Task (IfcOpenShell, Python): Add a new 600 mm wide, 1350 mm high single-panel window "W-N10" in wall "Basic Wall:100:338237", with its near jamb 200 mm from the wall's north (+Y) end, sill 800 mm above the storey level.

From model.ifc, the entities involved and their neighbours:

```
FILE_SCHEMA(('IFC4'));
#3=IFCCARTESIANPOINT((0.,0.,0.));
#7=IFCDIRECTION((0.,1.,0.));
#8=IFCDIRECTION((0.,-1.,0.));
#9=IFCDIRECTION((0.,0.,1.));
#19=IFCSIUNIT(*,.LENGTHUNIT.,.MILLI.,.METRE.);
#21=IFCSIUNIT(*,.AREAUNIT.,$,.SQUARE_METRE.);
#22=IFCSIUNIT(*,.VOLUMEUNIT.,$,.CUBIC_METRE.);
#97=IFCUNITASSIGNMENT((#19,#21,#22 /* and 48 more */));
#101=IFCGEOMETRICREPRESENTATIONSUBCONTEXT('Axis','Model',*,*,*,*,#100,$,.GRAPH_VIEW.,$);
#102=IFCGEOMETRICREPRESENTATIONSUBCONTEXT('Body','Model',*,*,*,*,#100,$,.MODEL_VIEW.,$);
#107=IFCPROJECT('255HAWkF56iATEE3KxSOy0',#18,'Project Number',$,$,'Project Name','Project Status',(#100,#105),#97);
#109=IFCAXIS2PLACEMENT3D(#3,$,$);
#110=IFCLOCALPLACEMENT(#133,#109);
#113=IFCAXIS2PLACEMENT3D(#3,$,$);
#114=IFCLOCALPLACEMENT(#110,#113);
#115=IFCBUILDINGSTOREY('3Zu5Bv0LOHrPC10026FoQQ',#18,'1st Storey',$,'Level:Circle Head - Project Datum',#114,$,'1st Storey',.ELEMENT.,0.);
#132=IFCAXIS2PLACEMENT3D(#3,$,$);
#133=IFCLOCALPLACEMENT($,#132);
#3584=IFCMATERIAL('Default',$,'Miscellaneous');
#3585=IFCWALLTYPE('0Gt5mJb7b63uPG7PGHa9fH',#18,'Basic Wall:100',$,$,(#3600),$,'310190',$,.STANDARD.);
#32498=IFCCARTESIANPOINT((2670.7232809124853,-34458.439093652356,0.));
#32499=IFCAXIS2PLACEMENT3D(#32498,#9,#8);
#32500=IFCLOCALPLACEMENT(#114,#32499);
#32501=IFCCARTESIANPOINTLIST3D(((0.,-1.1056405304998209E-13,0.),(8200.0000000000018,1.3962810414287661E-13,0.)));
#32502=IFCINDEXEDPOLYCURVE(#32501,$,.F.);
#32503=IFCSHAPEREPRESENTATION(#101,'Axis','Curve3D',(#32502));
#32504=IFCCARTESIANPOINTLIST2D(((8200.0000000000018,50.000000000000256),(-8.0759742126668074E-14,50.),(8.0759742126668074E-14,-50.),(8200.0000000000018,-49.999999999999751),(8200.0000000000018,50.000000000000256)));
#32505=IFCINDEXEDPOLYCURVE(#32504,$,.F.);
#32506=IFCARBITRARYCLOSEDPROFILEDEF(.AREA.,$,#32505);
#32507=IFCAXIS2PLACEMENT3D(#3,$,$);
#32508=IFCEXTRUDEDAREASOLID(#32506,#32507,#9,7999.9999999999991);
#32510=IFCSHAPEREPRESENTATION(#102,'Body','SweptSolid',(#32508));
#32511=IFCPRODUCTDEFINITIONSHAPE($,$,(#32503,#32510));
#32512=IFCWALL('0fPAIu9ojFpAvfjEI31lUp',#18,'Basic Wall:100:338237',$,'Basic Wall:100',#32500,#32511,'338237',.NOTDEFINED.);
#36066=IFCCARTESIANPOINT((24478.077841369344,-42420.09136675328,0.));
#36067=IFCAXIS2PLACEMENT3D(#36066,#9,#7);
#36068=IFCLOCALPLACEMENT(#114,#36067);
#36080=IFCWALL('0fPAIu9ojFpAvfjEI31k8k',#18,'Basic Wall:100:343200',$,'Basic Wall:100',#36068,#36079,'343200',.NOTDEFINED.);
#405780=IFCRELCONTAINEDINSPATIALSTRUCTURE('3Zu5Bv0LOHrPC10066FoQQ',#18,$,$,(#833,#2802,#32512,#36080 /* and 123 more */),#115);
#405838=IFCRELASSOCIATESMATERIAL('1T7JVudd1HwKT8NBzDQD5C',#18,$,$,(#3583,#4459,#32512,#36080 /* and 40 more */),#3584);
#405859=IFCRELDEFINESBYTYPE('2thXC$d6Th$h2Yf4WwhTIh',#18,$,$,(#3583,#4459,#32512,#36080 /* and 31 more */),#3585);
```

```python
import numpy as np
import ifcopenshell
import ifcopenshell.api.feature
import ifcopenshell.api.geometry
import ifcopenshell.api.root
import ifcopenshell.api.spatial
import ifcopenshell.geom
import ifcopenshell.util.element
import ifcopenshell.util.placement
import ifcopenshell.util.representation
import ifcopenshell.util.shape
import ifcopenshell.util.unit

model = ifcopenshell.open("model.ifc")
unit_scale = ifcopenshell.util.unit.calculate_unit_scale(model)
settings = ifcopenshell.geom.settings()


def volume(element):
    """Net volume in cubic metres, openings subtracted."""
    shape = ifcopenshell.geom.create_shape(settings, element)
    return ifcopenshell.util.shape.get_volume(shape.geometry)


wall = model.by_guid("0fPAIu9ojFpAvfjEI31lUp")
storey = ifcopenshell.util.element.get_container(wall, ifc_class="IfcBuildingStorey")
context = ifcopenshell.util.representation.get_context(model, "Model", "Body", "MODEL_VIEW")
before = volume(wall)

width, height, from_end, sill = 0.6, 1.35, 0.2, 0.8  # metres

# The wall runs along its own X axis, and the end named is its -X end.
wall_shape = ifcopenshell.geom.create_shape(settings, wall)
x, y, z = ifcopenshell.util.shape.get_vertices(wall_shape.geometry).T
start = x.min() + from_end
face, thickness = float(y.min()), float(y.max() - y.min())
wall_matrix = ifcopenshell.util.placement.get_local_placement(wall.ObjectPlacement)
level = ifcopenshell.util.placement.get_local_placement(storey.ObjectPlacement)[2, 3]


def in_wall(x, y):
    """Placement at x, y metres in the wall's axes, at sill height."""
    matrix = wall_matrix.copy()
    matrix[:, 3] = wall_matrix @ np.array([x / unit_scale, y / unit_scale, 0.0, 1.0])
    matrix[2, 3] = level + sill / unit_scale
    return matrix


# Opening: a box that overshoots both wall faces by 50 mm.
opening = ifcopenshell.api.root.create_entity(model, ifc_class="IfcOpeningElement", predefined_type="OPENING")
box = ifcopenshell.api.geometry.add_wall_representation(
    model, context=context, length=width, height=height, thickness=thickness + 0.1
)
ifcopenshell.api.geometry.assign_representation(model, product=opening, representation=box)
ifcopenshell.api.geometry.edit_object_placement(model, product=opening, matrix=in_wall(start, face - 0.05), is_si=False)
ifcopenshell.api.feature.add_feature(model, feature=opening, element=wall)

window = ifcopenshell.api.root.create_entity(model, ifc_class="IfcWindow", name="W-N10", predefined_type="WINDOW")
window.OverallWidth, window.OverallHeight = width / unit_scale, height / unit_scale
window.PartitioningType = "SINGLE_PANEL"
body = ifcopenshell.api.geometry.add_window_representation(
    model,
    context=context,
    overall_width=window.OverallWidth,
    overall_height=window.OverallHeight,
    partition_type="SINGLE_PANEL",
)
ifcopenshell.api.geometry.assign_representation(model, product=window, representation=body)
ifcopenshell.api.spatial.assign_container(model, products=[window], relating_structure=storey)
ifcopenshell.api.feature.add_filling(model, opening=opening, element=window)

# Centre the window in the wall's thickness.
ifcopenshell.api.geometry.edit_object_placement(model, product=window, matrix=in_wall(start, face), is_si=False)
window_shape = ifcopenshell.geom.create_shape(settings, window)
depth = ifcopenshell.util.shape.get_vertices(window_shape.geometry)[:, 1]
offset = face + thickness / 2 - (depth.min() + depth.max()) / 2
ifcopenshell.api.geometry.edit_object_placement(model, product=window, matrix=in_wall(start, offset), is_si=False)

after = volume(wall)

print(f"wall volume {before:.3f} -> {after:.3f} m3")

model.write("model_edited.ifc")
```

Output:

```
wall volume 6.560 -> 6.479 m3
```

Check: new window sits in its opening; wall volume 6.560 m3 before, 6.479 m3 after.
